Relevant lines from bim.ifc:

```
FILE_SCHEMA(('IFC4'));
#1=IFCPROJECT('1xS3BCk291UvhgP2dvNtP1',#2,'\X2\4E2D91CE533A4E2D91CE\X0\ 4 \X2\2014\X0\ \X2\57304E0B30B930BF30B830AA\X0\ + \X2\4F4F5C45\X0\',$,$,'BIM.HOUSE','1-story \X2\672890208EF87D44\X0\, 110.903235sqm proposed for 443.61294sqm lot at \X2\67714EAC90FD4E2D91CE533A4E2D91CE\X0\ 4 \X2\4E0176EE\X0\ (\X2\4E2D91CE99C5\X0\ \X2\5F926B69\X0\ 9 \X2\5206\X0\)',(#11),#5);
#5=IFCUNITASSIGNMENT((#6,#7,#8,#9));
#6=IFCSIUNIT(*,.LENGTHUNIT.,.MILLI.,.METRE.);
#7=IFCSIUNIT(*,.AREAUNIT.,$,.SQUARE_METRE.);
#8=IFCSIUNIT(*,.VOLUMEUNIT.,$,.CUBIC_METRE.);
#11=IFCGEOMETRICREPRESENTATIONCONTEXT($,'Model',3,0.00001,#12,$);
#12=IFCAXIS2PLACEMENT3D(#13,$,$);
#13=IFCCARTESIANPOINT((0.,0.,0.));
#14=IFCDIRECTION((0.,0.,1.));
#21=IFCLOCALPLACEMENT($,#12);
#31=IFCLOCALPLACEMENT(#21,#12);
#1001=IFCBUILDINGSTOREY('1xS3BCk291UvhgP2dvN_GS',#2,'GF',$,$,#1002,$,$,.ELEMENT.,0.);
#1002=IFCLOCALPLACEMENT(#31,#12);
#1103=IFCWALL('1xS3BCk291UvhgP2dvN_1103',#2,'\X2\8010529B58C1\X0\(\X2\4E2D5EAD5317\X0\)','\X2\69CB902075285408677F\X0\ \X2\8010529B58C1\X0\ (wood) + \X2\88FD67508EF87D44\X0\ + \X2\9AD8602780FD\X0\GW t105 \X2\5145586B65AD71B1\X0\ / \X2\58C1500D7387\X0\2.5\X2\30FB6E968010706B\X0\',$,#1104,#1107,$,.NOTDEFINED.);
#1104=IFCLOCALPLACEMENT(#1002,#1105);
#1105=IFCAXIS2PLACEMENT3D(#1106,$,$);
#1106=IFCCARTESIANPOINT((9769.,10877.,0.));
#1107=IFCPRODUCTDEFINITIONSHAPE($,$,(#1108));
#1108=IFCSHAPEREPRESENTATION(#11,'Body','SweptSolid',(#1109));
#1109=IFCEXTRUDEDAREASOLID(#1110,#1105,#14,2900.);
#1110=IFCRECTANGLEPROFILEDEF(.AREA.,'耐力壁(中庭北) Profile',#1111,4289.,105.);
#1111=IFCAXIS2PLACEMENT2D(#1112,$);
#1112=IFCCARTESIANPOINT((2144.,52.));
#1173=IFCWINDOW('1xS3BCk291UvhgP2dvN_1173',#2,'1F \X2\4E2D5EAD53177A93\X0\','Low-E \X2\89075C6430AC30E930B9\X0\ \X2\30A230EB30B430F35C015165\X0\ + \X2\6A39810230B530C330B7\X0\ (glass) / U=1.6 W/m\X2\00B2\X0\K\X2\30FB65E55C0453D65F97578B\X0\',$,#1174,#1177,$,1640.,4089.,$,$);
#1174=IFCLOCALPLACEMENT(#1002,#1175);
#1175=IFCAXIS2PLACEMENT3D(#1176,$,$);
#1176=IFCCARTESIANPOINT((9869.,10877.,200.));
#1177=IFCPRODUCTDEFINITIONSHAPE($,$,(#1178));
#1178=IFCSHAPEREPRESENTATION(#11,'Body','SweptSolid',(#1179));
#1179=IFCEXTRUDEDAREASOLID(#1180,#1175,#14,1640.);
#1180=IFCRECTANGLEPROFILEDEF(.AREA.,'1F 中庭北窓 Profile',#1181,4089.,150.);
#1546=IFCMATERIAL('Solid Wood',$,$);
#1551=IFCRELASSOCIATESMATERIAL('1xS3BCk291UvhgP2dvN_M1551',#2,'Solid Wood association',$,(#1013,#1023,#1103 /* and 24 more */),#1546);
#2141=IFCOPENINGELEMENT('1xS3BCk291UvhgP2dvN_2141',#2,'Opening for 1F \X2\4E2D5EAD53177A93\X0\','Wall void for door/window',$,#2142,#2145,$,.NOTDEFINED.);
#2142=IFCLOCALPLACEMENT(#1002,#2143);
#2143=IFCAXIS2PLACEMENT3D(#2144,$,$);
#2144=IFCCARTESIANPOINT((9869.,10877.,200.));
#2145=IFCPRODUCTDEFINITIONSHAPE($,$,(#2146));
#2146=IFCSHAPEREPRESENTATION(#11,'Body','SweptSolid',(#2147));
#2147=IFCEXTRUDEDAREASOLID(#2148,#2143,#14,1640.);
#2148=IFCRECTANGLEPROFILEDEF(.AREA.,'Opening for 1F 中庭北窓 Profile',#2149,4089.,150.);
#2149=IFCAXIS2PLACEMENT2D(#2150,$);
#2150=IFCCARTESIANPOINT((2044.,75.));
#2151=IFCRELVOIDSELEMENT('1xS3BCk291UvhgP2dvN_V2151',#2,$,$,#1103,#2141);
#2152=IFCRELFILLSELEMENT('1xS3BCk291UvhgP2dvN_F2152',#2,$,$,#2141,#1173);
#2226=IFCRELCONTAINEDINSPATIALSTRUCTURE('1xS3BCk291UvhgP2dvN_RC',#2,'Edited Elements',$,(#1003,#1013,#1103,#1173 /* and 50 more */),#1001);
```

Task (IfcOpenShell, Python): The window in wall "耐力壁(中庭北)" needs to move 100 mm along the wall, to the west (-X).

```python
import ifcopenshell
import ifcopenshell.api.geometry
import ifcopenshell.util.placement

model = ifcopenshell.open("bim.ifc")

window = model.by_guid("1xS3BCk291UvhgP2dvN_1173")
opening = window.FillsVoids[0].RelatingOpeningElement
wall = opening.VoidsElements[0].RelatingBuildingElement

wall_matrix = ifcopenshell.util.placement.get_local_placement(wall.ObjectPlacement)
shift = wall_matrix[:3, 0] * -100.0
before = ifcopenshell.util.placement.get_local_placement(window.ObjectPlacement)[:3, 3].copy()

# The window is not placed relative to its opening, so move both.
for product in (opening, window):
    matrix = ifcopenshell.util.placement.get_local_placement(product.ObjectPlacement)
    matrix[:3, 3] += shift
    ifcopenshell.api.geometry.edit_object_placement(model, product=product, matrix=matrix, is_si=False)

after = ifcopenshell.util.placement.get_local_placement(window.ObjectPlacement)[:3, 3]
print("window moved by", (after - before).round(3) + 0.0)

model.write("bim_edited.ifc")
```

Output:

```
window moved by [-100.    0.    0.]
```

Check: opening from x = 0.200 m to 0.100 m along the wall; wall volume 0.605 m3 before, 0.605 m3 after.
